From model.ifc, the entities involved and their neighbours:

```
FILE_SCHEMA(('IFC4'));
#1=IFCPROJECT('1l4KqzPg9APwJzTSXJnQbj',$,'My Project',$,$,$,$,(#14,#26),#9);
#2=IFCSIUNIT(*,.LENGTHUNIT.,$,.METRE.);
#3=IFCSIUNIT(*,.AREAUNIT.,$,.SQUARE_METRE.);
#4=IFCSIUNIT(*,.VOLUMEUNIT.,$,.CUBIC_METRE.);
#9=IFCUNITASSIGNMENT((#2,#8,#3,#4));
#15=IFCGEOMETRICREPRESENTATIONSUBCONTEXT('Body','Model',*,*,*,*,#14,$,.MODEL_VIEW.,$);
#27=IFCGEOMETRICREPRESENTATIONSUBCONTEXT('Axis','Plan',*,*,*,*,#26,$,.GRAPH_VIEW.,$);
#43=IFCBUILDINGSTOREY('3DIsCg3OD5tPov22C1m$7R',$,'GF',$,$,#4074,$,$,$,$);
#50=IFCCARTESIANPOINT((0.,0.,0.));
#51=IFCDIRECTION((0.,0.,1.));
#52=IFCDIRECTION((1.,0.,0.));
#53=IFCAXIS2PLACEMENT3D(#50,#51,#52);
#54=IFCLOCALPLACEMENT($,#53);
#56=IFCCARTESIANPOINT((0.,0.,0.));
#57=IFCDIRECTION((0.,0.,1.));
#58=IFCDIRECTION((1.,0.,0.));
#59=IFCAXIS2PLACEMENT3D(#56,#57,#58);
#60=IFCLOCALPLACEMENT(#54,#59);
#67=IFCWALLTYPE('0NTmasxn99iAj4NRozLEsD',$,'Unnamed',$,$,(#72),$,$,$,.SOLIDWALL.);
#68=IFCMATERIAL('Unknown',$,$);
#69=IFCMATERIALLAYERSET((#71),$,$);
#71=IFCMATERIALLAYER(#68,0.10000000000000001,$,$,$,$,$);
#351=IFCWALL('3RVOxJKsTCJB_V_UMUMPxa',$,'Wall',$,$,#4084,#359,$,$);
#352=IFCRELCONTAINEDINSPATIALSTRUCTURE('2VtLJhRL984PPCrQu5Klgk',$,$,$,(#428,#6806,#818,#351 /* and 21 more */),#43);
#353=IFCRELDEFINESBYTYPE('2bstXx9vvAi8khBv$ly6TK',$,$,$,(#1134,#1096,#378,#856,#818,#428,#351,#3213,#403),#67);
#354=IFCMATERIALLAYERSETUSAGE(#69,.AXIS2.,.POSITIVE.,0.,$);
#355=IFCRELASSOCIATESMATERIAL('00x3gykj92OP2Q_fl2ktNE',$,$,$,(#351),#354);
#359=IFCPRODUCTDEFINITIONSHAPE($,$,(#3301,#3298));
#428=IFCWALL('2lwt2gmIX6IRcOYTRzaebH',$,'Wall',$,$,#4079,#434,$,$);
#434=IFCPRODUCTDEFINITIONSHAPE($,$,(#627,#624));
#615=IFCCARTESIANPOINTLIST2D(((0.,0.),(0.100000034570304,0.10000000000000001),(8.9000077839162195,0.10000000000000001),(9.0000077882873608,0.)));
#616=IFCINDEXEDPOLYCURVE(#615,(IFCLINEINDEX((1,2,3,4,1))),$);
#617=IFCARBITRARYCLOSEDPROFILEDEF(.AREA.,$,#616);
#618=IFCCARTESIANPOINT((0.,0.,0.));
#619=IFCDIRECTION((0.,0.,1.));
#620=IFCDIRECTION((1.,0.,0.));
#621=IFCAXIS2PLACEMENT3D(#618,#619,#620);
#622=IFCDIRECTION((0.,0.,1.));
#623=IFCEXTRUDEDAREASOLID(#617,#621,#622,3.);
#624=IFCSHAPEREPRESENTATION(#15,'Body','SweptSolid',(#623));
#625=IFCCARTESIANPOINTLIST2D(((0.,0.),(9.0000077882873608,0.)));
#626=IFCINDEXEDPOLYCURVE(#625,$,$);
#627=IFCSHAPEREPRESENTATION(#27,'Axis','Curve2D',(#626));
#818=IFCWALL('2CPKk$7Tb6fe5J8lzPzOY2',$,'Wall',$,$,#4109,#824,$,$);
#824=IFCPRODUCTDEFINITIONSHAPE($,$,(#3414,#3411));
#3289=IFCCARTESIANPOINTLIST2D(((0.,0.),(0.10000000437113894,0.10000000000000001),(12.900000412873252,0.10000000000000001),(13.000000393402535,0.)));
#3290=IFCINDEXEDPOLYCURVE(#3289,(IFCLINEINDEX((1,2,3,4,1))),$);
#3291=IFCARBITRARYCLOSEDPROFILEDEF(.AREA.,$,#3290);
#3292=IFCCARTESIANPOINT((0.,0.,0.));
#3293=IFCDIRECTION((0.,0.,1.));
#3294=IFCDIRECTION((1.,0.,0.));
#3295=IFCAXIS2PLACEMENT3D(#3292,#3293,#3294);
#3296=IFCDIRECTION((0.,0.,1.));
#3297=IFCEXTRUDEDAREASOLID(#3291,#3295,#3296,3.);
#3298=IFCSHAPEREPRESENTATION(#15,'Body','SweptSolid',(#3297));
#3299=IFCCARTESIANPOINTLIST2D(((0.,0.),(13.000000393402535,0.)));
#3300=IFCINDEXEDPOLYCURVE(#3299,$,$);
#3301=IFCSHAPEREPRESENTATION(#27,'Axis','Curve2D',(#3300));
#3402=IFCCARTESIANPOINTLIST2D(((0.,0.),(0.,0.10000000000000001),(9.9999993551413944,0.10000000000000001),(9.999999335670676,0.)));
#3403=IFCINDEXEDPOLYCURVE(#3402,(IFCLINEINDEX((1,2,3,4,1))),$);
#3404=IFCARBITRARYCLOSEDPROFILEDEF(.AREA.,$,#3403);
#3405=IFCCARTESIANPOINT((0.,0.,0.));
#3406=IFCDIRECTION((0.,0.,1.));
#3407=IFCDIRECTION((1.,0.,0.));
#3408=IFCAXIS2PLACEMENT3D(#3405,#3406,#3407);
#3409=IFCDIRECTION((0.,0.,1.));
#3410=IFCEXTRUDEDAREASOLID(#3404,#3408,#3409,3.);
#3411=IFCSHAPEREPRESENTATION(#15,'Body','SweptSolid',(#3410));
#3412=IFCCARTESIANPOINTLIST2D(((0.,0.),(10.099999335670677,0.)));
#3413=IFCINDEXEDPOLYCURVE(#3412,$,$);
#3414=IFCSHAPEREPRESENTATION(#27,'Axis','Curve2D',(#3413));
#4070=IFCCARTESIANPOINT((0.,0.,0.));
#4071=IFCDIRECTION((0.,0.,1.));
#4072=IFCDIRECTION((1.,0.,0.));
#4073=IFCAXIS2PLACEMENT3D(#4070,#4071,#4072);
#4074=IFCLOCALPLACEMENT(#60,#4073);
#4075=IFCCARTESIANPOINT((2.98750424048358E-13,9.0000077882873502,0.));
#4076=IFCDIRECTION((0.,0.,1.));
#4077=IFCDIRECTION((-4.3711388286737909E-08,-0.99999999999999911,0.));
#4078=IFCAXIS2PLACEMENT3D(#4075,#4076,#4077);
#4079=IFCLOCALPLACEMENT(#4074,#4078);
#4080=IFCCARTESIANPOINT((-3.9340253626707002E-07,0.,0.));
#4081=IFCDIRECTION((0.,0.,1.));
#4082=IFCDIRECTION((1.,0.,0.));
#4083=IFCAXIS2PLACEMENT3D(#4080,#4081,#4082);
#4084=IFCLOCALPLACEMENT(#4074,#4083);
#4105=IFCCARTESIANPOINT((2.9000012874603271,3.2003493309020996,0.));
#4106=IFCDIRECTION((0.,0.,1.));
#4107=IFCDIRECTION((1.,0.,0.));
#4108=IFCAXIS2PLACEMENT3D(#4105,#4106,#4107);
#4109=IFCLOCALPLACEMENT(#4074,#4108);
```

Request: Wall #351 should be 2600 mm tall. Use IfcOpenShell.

```python
import ifcopenshell
import ifcopenshell.geom
import ifcopenshell.util.representation
import ifcopenshell.util.shape
import ifcopenshell.util.unit

model = ifcopenshell.open("model.ifc")
unit_scale = ifcopenshell.util.unit.calculate_unit_scale(model)
settings = ifcopenshell.geom.settings()


def volume(element):
    """Net volume in cubic metres, openings subtracted."""
    shape = ifcopenshell.geom.create_shape(settings, element)
    return ifcopenshell.util.shape.get_volume(shape.geometry)


wall = model.by_guid("3RVOxJKsTCJB_V_UMUMPxa")
before = volume(wall)

body = ifcopenshell.util.representation.get_representation(wall, "Model", "Body")
solid = body.Items[0]
old_height = solid.Depth
solid.Depth = 2.6 / unit_scale
after = volume(wall)

print(f"height {old_height:g} -> {solid.Depth:g}, volume {before:.3f} -> {after:.3f} m3")

model.write("model_v2.ifc")
```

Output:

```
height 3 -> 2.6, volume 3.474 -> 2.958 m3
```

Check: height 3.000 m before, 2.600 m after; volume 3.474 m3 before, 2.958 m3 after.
